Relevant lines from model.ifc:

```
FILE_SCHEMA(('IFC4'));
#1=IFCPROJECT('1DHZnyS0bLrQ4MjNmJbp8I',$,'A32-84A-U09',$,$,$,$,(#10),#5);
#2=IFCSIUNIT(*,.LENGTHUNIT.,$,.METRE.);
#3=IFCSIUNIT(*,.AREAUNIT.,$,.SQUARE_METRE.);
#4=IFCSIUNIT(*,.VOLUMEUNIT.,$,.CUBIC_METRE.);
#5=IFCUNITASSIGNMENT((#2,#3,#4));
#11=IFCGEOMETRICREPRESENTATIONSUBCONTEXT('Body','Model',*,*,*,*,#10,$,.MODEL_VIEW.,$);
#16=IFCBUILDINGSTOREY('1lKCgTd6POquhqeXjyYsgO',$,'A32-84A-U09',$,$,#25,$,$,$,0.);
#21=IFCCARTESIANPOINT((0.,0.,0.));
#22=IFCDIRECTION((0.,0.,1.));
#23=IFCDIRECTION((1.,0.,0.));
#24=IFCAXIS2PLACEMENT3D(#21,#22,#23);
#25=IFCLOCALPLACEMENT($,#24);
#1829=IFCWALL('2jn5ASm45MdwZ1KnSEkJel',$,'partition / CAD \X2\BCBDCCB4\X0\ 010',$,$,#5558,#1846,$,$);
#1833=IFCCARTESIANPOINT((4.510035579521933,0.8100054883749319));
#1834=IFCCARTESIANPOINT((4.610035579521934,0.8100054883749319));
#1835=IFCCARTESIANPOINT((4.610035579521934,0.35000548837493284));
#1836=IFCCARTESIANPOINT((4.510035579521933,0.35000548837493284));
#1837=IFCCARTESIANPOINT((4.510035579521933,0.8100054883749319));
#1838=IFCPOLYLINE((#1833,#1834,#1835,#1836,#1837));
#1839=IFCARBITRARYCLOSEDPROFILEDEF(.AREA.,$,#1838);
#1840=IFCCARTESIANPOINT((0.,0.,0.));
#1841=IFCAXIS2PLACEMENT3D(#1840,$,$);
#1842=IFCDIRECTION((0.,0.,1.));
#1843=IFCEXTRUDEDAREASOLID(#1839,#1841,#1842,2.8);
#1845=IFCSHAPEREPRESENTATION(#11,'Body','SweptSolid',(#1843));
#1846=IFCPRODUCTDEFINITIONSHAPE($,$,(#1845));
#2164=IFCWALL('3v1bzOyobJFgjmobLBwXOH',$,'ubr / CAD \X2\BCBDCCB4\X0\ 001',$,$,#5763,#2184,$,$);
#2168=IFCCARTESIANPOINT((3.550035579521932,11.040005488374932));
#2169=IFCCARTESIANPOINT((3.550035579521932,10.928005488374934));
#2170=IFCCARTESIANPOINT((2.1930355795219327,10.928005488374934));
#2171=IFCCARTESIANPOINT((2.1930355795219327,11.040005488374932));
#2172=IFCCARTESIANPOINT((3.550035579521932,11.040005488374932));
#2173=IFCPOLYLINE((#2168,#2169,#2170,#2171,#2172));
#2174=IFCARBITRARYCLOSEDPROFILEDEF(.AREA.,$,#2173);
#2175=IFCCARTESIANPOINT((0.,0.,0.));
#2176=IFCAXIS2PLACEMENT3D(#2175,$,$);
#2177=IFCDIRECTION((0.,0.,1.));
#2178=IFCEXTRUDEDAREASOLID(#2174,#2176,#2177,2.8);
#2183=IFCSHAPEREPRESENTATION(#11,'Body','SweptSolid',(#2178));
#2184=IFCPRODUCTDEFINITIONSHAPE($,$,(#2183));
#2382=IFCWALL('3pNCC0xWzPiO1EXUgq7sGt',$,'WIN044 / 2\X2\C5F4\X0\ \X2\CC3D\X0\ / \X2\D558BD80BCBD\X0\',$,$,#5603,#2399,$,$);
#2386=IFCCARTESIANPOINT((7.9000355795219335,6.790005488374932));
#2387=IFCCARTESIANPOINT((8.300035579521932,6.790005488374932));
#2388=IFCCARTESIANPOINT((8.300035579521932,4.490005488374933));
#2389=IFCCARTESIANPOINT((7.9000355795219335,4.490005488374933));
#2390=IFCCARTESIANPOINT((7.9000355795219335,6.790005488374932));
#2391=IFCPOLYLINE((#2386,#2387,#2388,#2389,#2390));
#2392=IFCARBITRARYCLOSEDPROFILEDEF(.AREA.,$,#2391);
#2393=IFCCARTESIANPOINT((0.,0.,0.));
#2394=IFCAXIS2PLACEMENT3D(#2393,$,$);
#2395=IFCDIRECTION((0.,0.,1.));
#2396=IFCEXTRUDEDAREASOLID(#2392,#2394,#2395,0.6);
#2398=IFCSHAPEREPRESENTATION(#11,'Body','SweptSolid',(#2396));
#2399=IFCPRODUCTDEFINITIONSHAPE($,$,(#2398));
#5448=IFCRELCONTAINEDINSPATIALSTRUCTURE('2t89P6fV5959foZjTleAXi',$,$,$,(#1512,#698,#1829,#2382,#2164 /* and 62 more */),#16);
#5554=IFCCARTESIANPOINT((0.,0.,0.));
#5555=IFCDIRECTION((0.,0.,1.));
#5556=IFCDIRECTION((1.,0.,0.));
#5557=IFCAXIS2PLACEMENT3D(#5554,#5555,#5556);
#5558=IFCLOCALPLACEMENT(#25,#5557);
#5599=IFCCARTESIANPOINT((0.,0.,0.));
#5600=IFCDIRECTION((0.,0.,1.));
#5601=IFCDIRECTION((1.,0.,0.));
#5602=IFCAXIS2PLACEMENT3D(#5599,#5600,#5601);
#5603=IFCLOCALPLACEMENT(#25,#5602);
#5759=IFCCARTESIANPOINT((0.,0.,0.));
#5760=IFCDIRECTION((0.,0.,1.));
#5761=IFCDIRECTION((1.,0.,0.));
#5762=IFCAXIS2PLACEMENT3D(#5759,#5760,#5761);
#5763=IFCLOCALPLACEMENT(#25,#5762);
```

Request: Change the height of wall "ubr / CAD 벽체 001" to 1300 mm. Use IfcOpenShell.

```python
import ifcopenshell
import ifcopenshell.geom
import ifcopenshell.util.representation
import ifcopenshell.util.shape
import ifcopenshell.util.unit

model = ifcopenshell.open("model.ifc")
unit_scale = ifcopenshell.util.unit.calculate_unit_scale(model)
settings = ifcopenshell.geom.settings()


def volume(element):
    """Net volume in cubic metres, openings subtracted."""
    shape = ifcopenshell.geom.create_shape(settings, element)
    return ifcopenshell.util.shape.get_volume(shape.geometry)


wall = model.by_guid("3v1bzOyobJFgjmobLBwXOH")
before = volume(wall)

body = ifcopenshell.util.representation.get_representation(wall, "Model", "Body")
solid = body.Items[0]
old_height = solid.Depth
solid.Depth = 1.3 / unit_scale
after = volume(wall)

print(f"height {old_height:g} -> {solid.Depth:g}, volume {before:.3f} -> {after:.3f} m3")

model.write("model_updated.ifc")
```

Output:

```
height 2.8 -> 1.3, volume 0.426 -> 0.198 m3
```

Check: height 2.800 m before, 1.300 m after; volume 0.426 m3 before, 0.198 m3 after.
